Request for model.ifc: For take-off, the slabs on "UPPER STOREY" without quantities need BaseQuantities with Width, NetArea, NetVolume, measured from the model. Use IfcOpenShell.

First a look at what the model holds.

```python
import ifcopenshell
import ifcopenshell.util.element
import ifcopenshell.util.unit

model = ifcopenshell.open("model.ifc")
print(model.schema)
for unit_type in ("LENGTHUNIT", "AREAUNIT", "VOLUMEUNIT"):
    print(unit_type, ifcopenshell.util.unit.calculate_unit_scale(model, unit_type))
storey = next(s for s in model.by_type("IfcBuildingStorey") if s.Name == "UPPER STOREY")
slabs = [e for e in ifcopenshell.util.element.get_decomposition(storey) if e.is_a("IfcSlab")]
for e in sorted(slabs, key=lambda e: e.id()):
    print(e.id(), e.is_a(), e.Name, list(ifcopenshell.util.element.get_psets(e, qtos_only=True)), sep=" | ")
```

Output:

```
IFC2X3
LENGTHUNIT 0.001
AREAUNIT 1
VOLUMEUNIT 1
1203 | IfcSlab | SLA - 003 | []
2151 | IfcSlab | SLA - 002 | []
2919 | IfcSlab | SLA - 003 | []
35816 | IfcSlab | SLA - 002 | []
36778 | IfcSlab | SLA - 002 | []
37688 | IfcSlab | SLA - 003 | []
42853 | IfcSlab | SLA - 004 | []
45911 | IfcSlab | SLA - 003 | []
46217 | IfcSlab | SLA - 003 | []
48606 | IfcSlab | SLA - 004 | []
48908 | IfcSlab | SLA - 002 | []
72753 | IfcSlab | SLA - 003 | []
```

```python
import ifcopenshell
import ifcopenshell.api.pset
import ifcopenshell.geom
import ifcopenshell.util.element
import ifcopenshell.util.shape
import ifcopenshell.util.unit

model = ifcopenshell.open("model.ifc")
unit_scale = ifcopenshell.util.unit.calculate_unit_scale(model)
area_scale = ifcopenshell.util.unit.calculate_unit_scale(model, "AREAUNIT")
volume_scale = ifcopenshell.util.unit.calculate_unit_scale(model, "VOLUMEUNIT")
settings = ifcopenshell.geom.settings()

storey = next(s for s in model.by_type("IfcBuildingStorey") if s.Name == "UPPER STOREY")
slabs = [e for e in ifcopenshell.util.element.get_decomposition(storey) if e.is_a("IfcSlab")]

for e in sorted(slabs, key=lambda e: e.id()):
    if ifcopenshell.util.element.get_psets(e, qtos_only=True, should_inherit=False):
        continue
    # Geometry comes back in metres, in the element's own axes.
    shape = ifcopenshell.geom.create_shape(settings, e)
    values = {
        "Width": ifcopenshell.util.shape.get_z(shape.geometry) / unit_scale,
        "NetArea": ifcopenshell.util.shape.get_footprint_area(shape.geometry) / area_scale,
        "NetVolume": ifcopenshell.util.shape.get_volume(shape.geometry) / volume_scale,
    }
    qto = ifcopenshell.api.pset.add_qto(model, product=e, name="BaseQuantities")
    ifcopenshell.api.pset.edit_qto(model, qto=qto, properties=values)
    print(e.id(), {k: round(v, 3) for k, v in values.items()})

model.write("model-out.ifc")
```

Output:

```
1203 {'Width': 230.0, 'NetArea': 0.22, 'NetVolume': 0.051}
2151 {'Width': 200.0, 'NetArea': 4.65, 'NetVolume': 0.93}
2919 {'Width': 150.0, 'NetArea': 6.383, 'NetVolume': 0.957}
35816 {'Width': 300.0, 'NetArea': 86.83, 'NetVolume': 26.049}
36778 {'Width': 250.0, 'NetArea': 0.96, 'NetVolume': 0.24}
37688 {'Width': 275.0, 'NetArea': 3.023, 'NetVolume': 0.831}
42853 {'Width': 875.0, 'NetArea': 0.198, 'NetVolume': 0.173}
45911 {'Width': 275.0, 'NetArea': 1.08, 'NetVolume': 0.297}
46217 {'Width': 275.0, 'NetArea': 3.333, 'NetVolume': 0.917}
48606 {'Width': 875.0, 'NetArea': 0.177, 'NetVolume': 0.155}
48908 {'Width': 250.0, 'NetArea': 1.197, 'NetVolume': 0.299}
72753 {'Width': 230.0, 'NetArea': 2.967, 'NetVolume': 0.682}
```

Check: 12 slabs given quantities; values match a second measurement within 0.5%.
